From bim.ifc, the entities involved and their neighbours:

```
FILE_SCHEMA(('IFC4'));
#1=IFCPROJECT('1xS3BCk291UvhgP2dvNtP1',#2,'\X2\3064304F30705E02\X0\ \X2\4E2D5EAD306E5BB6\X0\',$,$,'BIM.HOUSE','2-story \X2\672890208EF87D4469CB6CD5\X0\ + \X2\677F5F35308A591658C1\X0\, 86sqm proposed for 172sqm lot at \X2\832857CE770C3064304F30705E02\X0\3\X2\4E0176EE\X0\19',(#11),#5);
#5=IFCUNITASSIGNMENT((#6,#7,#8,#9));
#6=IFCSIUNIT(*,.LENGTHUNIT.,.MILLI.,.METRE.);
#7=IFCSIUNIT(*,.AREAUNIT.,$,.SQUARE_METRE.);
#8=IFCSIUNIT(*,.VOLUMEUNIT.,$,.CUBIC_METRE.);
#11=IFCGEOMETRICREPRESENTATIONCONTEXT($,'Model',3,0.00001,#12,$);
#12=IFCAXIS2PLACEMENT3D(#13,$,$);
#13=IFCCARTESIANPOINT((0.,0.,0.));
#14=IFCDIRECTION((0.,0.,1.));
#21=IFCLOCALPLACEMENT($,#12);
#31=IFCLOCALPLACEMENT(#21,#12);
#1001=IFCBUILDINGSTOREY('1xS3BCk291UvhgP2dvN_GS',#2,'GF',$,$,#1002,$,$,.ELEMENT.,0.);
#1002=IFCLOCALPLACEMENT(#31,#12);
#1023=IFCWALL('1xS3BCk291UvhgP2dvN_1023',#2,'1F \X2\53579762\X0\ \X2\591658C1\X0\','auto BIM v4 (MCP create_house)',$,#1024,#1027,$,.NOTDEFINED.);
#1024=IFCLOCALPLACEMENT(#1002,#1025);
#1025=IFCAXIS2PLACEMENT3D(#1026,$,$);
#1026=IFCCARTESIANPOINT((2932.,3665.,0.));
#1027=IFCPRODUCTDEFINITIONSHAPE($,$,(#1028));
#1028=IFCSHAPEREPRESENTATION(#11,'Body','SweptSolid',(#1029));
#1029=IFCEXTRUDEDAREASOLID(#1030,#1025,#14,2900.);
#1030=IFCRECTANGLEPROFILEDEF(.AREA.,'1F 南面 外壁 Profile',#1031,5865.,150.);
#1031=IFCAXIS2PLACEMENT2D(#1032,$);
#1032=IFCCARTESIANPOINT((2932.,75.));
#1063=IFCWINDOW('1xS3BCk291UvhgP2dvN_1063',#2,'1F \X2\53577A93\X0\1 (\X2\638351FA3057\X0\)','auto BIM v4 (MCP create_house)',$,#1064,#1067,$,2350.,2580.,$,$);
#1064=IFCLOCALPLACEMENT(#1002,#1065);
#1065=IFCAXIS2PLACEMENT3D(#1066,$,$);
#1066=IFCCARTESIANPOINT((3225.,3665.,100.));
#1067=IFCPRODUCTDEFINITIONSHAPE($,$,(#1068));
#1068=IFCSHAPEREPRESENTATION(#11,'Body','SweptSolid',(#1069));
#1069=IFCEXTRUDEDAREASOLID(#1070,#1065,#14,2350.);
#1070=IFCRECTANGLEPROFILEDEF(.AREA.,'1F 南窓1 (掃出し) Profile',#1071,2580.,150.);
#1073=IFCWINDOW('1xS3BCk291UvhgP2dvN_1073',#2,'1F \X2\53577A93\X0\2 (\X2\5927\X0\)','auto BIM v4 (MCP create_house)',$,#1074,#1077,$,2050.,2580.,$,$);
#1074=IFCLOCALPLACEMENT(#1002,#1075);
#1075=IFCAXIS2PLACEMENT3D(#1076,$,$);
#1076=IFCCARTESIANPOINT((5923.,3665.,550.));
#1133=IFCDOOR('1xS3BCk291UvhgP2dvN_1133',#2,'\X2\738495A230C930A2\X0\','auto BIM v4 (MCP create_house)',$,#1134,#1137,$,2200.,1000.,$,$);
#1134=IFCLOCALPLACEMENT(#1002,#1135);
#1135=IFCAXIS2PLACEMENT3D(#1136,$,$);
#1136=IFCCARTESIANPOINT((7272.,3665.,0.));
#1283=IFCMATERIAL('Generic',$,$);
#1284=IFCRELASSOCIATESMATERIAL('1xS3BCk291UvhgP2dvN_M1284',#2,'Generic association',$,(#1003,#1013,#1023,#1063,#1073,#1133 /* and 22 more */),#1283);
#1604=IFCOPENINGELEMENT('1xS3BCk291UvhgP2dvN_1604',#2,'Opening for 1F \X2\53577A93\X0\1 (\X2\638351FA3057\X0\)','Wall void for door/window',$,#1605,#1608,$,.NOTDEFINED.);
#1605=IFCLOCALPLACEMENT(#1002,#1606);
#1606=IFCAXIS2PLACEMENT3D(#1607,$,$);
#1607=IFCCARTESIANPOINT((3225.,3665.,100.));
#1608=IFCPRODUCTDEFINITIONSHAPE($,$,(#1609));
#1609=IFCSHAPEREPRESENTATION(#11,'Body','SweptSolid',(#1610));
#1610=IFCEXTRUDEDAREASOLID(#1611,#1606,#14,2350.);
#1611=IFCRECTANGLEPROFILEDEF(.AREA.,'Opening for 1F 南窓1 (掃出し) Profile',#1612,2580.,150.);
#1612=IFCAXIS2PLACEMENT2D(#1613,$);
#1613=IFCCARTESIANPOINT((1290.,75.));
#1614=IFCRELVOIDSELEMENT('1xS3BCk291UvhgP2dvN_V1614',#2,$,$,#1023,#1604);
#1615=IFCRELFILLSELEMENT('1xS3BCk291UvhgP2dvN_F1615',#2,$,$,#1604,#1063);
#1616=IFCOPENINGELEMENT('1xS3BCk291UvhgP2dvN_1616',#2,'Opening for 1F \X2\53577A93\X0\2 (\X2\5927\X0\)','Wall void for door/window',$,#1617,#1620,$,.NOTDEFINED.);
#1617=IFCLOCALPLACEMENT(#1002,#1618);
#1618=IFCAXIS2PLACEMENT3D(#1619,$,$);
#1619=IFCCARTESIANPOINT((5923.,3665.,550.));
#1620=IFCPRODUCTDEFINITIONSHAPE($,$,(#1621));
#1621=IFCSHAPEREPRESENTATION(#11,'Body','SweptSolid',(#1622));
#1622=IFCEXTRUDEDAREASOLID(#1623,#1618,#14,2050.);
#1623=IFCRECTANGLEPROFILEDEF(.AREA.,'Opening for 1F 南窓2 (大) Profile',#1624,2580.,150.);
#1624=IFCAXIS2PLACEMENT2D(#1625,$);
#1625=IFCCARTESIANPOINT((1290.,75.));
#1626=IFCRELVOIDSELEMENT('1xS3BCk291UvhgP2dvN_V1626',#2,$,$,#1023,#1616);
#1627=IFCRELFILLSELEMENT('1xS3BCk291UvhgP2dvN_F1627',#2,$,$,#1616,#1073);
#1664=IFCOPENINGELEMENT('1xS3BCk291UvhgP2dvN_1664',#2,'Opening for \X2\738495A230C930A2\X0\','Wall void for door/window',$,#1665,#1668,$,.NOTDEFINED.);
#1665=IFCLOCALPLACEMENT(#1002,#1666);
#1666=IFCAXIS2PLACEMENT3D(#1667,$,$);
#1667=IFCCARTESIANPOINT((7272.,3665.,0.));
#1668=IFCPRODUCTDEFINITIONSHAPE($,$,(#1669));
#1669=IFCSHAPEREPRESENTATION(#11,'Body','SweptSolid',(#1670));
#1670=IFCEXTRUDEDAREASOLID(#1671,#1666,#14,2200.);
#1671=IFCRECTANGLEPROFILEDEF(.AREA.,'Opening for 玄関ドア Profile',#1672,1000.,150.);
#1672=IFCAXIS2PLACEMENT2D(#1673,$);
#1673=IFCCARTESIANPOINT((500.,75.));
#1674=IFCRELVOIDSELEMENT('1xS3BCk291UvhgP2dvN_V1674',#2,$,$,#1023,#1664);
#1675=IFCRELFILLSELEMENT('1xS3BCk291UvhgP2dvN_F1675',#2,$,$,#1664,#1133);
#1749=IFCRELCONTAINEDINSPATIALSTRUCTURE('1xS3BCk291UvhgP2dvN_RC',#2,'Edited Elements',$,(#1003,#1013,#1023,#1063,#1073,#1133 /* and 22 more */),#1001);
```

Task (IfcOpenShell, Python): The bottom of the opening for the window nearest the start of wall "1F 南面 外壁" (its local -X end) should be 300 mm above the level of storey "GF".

```python
import numpy as np
import ifcopenshell
import ifcopenshell.api.geometry
import ifcopenshell.geom
import ifcopenshell.util.element
import ifcopenshell.util.placement
import ifcopenshell.util.shape
import ifcopenshell.util.unit

model = ifcopenshell.open("bim.ifc")
unit_scale = ifcopenshell.util.unit.calculate_unit_scale(model)

window = model.by_guid("1xS3BCk291UvhgP2dvN_1063")
opening = window.FillsVoids[0].RelatingOpeningElement
storey = ifcopenshell.util.element.get_container(window, ifc_class="IfcBuildingStorey")
level = ifcopenshell.util.placement.get_local_placement(storey.ObjectPlacement)[2, 3]

# The opening's origin need not be at the sill, so measure its lowest point.
shape = ifcopenshell.geom.create_shape(ifcopenshell.geom.settings(), opening)
bottom = ifcopenshell.util.shape.get_shape_bottom_elevation(shape, shape.geometry) / unit_scale
dz = level + 0.3 / unit_scale - bottom

shift = np.array([0.0, 0.0, dz])
# The window is not placed relative to its opening, so move both.
for product in (opening, window):
    matrix = ifcopenshell.util.placement.get_local_placement(product.ObjectPlacement)
    matrix[:3, 3] += shift
    ifcopenshell.api.geometry.edit_object_placement(model, product=product, matrix=matrix, is_si=False)

print(f"moved by {dz * unit_scale:+.3f} m")

model.write("bim_edited.ifc")
```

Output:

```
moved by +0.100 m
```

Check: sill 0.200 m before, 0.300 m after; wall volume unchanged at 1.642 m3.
